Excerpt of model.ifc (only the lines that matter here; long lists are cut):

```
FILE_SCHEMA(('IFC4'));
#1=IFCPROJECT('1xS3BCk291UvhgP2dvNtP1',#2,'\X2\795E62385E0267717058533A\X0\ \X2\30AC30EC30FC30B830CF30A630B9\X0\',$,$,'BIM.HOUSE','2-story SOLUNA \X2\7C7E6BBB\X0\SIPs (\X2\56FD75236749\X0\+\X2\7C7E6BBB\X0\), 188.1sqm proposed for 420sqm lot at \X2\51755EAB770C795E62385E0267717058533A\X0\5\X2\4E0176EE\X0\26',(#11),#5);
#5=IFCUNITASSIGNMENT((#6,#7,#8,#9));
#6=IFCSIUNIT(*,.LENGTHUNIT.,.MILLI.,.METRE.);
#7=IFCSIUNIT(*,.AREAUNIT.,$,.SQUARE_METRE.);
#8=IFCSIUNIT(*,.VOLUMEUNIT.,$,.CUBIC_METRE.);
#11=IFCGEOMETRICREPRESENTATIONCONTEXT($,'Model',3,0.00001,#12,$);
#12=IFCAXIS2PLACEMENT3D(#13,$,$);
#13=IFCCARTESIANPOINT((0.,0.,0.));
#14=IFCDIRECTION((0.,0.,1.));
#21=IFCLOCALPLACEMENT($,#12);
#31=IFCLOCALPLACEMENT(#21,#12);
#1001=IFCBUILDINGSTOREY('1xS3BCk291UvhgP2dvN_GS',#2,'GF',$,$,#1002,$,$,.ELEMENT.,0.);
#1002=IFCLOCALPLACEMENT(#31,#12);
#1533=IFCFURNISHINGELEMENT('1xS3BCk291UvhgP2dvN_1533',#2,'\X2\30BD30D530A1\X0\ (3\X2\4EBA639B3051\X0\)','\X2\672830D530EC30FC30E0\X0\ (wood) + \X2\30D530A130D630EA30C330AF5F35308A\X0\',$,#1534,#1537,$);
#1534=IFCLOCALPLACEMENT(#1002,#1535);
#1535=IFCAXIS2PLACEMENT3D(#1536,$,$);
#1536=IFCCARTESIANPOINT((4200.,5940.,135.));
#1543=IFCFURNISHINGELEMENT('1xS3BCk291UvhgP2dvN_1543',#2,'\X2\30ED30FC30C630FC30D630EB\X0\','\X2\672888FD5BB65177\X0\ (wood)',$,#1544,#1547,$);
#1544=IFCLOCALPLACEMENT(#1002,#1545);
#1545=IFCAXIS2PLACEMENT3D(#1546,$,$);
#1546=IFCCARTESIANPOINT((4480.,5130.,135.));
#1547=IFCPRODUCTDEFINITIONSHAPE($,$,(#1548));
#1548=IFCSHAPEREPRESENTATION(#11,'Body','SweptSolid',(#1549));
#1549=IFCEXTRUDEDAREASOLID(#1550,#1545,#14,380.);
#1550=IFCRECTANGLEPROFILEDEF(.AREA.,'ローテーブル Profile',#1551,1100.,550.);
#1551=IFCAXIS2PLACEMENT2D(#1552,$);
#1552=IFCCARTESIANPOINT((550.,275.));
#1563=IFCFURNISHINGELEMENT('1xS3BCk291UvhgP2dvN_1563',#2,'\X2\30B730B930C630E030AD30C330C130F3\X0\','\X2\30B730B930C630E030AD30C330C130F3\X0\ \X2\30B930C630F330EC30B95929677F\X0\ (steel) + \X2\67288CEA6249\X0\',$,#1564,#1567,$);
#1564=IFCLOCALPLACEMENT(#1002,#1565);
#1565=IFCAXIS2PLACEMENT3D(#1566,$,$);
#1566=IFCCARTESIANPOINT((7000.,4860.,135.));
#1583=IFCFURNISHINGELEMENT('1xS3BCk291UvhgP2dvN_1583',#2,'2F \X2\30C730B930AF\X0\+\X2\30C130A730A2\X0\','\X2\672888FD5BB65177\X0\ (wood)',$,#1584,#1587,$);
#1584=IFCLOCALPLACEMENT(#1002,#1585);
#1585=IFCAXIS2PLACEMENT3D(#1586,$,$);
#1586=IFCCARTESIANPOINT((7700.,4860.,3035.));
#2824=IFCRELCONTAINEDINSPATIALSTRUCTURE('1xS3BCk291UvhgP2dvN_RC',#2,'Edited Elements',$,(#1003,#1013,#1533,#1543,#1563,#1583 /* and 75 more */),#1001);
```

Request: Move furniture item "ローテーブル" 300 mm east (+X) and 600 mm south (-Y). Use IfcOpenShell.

```python
import ifcopenshell
import ifcopenshell.api.geometry
import ifcopenshell.util.placement
import ifcopenshell.util.unit

model = ifcopenshell.open("model.ifc")
unit_scale = ifcopenshell.util.unit.calculate_unit_scale(model)

item = model.by_guid("1xS3BCk291UvhgP2dvN_1543")
matrix = ifcopenshell.util.placement.get_local_placement(item.ObjectPlacement)
matrix[0, 3] += 0.3 / unit_scale
matrix[1, 3] -= 0.6 / unit_scale
ifcopenshell.api.geometry.edit_object_placement(model, product=item, matrix=matrix, is_si=False)

print(ifcopenshell.util.placement.get_local_placement(item.ObjectPlacement).round(3) + 0.0)

model.write("model_rev.ifc")
```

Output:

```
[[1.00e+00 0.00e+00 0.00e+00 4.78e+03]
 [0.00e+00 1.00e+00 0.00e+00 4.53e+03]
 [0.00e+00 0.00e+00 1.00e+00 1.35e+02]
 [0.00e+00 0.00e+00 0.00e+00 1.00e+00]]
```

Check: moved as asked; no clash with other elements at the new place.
